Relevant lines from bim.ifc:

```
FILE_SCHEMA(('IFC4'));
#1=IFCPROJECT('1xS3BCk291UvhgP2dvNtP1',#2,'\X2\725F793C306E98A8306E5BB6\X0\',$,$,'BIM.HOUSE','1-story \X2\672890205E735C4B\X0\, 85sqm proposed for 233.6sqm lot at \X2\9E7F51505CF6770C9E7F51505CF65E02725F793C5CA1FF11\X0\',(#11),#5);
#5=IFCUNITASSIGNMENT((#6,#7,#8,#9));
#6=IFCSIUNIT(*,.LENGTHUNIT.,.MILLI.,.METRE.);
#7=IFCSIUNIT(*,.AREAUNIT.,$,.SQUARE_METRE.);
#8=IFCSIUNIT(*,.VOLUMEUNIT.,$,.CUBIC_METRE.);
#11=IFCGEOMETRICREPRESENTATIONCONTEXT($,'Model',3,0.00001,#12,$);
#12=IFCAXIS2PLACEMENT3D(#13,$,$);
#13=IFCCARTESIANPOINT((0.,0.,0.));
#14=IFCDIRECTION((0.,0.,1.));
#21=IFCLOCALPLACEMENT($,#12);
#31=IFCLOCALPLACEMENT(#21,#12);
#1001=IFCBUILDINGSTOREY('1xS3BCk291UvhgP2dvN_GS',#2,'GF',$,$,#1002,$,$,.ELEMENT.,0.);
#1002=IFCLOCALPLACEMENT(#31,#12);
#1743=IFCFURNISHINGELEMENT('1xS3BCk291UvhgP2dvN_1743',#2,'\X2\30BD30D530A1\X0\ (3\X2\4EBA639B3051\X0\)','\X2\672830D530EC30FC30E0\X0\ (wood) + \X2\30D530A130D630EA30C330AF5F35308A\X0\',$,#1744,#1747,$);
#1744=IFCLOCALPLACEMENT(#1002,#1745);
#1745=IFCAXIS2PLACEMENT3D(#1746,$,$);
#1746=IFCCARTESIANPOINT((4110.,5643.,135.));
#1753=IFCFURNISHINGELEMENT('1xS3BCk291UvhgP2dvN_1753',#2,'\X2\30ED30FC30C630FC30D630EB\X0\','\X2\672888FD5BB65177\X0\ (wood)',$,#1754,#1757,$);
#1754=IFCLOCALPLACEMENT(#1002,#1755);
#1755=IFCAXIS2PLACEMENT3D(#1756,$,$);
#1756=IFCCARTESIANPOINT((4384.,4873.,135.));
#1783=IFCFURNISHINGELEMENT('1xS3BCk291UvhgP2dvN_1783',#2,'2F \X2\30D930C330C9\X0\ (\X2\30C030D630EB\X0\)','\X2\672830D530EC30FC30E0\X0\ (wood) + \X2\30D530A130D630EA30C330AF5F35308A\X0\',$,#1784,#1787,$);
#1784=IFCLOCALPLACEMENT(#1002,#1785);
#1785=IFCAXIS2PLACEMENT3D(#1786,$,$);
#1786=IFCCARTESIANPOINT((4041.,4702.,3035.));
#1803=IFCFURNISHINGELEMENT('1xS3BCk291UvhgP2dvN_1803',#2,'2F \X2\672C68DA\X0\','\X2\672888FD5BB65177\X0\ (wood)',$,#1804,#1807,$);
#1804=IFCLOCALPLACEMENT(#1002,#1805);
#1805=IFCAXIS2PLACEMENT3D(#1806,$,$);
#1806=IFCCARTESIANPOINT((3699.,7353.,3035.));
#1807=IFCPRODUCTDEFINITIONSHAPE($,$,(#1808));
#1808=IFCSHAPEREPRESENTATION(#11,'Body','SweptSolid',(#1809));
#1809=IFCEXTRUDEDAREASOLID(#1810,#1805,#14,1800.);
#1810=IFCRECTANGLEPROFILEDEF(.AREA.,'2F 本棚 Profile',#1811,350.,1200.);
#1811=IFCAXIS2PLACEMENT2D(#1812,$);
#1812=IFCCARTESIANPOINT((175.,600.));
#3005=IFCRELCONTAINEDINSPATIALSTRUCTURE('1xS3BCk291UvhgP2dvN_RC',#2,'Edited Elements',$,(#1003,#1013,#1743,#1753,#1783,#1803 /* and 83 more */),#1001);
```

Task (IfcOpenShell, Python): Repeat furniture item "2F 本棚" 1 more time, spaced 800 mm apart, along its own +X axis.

```python
import ifcopenshell
import ifcopenshell.api.geometry
import ifcopenshell.api.root
import ifcopenshell.util.element
import ifcopenshell.util.placement
import ifcopenshell.util.unit

model = ifcopenshell.open("bim.ifc")
unit_scale = ifcopenshell.util.unit.calculate_unit_scale(model)


def reuse_history(source, copy):
    """copy_class also copies each property set's owner history, people and application; keep the originals."""
    for rel in copy.IsDefinedBy:
        if rel.is_a("IfcRelDefinesByProperties") and (history := rel.RelatingPropertyDefinition.OwnerHistory):
            rel.RelatingPropertyDefinition.OwnerHistory = source.OwnerHistory
            ifcopenshell.util.element.remove_deep2(model, history)


source = model.by_id(1803)
base = ifcopenshell.util.placement.get_local_placement(source.ObjectPlacement)
step = base[:3, 0] * 0.8 / unit_scale

for i in range(1, 2):
    copy = ifcopenshell.api.root.copy_class(model, product=source)
    copy.Representation = ifcopenshell.util.element.copy_deep(
        model, source.Representation, exclude=["IfcGeometricRepresentationContext", "IfcRepresentationMap"]
    )
    reuse_history(source, copy)
    matrix = base.copy()
    matrix[:3, 3] += i * step
    print("added at", matrix[:3, 3].round(3) + 0.0)
    ifcopenshell.api.geometry.edit_object_placement(model, product=copy, matrix=matrix, is_si=False)

model.write("bim_updated.ifc")
```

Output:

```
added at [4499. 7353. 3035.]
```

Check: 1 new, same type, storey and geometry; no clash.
